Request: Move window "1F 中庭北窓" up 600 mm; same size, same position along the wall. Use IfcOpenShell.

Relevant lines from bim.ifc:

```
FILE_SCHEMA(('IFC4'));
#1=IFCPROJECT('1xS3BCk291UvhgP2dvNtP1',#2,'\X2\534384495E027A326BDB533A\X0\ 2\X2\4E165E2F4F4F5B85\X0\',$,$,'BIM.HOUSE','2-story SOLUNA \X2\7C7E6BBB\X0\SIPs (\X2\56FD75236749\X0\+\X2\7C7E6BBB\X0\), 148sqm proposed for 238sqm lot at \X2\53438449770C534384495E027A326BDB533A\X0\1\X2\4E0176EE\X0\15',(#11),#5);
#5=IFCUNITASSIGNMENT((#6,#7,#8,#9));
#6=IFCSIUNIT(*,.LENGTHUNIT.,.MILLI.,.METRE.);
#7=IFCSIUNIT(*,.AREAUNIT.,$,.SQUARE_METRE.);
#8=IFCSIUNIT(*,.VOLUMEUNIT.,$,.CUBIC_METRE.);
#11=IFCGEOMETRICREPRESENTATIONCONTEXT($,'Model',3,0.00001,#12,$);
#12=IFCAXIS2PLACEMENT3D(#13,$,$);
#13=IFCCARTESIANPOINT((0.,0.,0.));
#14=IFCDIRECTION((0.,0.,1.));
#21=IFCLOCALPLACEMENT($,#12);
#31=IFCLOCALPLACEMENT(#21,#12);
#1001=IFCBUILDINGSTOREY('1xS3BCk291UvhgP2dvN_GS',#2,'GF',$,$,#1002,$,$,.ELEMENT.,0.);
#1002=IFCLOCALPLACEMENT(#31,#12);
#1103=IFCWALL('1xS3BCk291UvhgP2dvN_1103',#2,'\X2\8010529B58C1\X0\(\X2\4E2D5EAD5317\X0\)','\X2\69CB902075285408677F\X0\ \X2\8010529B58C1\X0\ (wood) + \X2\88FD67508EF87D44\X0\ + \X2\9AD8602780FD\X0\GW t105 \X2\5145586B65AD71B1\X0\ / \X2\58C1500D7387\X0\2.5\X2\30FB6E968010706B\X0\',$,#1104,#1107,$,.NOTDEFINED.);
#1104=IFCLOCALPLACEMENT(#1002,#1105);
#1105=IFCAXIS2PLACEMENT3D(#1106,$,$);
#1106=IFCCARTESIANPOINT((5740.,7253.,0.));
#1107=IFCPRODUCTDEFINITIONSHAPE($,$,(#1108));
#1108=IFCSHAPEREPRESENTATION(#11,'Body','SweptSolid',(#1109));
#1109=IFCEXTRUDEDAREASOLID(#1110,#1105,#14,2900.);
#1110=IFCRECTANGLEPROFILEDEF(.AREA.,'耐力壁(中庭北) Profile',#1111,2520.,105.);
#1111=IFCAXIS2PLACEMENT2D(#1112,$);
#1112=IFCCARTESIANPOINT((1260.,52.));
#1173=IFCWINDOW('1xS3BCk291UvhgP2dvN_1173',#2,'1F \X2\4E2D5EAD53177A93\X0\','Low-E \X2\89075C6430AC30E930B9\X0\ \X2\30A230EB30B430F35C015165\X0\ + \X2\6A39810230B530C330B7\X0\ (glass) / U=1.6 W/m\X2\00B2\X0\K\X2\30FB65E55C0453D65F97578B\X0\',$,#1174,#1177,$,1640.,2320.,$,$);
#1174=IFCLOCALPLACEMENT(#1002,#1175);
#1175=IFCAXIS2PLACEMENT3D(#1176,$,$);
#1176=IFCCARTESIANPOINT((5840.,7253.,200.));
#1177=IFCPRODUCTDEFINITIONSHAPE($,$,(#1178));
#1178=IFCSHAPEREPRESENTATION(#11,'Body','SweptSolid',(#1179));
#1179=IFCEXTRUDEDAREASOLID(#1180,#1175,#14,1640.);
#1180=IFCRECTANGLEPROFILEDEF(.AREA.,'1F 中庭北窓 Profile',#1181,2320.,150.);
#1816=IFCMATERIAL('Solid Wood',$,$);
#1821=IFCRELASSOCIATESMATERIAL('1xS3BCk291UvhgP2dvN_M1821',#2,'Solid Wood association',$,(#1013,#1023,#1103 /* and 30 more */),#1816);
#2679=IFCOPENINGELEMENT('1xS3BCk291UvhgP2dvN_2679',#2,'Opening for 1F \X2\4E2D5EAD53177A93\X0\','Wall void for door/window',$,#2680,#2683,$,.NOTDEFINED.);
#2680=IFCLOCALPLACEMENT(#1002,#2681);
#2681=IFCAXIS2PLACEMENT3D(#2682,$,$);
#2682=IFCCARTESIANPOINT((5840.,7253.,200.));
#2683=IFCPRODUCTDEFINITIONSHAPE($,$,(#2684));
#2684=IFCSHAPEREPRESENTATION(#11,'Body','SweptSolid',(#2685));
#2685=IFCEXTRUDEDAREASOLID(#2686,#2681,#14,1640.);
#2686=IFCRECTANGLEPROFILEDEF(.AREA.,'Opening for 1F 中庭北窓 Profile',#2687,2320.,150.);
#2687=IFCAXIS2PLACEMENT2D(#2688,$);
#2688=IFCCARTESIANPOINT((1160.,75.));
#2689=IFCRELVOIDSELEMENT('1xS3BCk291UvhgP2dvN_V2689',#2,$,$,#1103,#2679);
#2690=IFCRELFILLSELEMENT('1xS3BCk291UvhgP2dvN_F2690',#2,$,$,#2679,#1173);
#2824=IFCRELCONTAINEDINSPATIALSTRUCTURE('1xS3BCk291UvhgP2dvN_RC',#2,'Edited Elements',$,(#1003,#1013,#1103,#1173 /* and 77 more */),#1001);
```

```python
import numpy as np
import ifcopenshell
import ifcopenshell.api.geometry
import ifcopenshell.util.placement
import ifcopenshell.util.unit

model = ifcopenshell.open("bim.ifc")
unit_scale = ifcopenshell.util.unit.calculate_unit_scale(model)

window = model.by_id(1173)
opening = window.FillsVoids[0].RelatingOpeningElement
dz = 0.6 / unit_scale

shift = np.array([0.0, 0.0, dz])
# The window is not placed relative to its opening, so move both.
for product in (opening, window):
    matrix = ifcopenshell.util.placement.get_local_placement(product.ObjectPlacement)
    matrix[:3, 3] += shift
    ifcopenshell.api.geometry.edit_object_placement(model, product=product, matrix=matrix, is_si=False)

print(f"moved by {dz * unit_scale:+.3f} m")

model.write("bim_edited.ifc")
```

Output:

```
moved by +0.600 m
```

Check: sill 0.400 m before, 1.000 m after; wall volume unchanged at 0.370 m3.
